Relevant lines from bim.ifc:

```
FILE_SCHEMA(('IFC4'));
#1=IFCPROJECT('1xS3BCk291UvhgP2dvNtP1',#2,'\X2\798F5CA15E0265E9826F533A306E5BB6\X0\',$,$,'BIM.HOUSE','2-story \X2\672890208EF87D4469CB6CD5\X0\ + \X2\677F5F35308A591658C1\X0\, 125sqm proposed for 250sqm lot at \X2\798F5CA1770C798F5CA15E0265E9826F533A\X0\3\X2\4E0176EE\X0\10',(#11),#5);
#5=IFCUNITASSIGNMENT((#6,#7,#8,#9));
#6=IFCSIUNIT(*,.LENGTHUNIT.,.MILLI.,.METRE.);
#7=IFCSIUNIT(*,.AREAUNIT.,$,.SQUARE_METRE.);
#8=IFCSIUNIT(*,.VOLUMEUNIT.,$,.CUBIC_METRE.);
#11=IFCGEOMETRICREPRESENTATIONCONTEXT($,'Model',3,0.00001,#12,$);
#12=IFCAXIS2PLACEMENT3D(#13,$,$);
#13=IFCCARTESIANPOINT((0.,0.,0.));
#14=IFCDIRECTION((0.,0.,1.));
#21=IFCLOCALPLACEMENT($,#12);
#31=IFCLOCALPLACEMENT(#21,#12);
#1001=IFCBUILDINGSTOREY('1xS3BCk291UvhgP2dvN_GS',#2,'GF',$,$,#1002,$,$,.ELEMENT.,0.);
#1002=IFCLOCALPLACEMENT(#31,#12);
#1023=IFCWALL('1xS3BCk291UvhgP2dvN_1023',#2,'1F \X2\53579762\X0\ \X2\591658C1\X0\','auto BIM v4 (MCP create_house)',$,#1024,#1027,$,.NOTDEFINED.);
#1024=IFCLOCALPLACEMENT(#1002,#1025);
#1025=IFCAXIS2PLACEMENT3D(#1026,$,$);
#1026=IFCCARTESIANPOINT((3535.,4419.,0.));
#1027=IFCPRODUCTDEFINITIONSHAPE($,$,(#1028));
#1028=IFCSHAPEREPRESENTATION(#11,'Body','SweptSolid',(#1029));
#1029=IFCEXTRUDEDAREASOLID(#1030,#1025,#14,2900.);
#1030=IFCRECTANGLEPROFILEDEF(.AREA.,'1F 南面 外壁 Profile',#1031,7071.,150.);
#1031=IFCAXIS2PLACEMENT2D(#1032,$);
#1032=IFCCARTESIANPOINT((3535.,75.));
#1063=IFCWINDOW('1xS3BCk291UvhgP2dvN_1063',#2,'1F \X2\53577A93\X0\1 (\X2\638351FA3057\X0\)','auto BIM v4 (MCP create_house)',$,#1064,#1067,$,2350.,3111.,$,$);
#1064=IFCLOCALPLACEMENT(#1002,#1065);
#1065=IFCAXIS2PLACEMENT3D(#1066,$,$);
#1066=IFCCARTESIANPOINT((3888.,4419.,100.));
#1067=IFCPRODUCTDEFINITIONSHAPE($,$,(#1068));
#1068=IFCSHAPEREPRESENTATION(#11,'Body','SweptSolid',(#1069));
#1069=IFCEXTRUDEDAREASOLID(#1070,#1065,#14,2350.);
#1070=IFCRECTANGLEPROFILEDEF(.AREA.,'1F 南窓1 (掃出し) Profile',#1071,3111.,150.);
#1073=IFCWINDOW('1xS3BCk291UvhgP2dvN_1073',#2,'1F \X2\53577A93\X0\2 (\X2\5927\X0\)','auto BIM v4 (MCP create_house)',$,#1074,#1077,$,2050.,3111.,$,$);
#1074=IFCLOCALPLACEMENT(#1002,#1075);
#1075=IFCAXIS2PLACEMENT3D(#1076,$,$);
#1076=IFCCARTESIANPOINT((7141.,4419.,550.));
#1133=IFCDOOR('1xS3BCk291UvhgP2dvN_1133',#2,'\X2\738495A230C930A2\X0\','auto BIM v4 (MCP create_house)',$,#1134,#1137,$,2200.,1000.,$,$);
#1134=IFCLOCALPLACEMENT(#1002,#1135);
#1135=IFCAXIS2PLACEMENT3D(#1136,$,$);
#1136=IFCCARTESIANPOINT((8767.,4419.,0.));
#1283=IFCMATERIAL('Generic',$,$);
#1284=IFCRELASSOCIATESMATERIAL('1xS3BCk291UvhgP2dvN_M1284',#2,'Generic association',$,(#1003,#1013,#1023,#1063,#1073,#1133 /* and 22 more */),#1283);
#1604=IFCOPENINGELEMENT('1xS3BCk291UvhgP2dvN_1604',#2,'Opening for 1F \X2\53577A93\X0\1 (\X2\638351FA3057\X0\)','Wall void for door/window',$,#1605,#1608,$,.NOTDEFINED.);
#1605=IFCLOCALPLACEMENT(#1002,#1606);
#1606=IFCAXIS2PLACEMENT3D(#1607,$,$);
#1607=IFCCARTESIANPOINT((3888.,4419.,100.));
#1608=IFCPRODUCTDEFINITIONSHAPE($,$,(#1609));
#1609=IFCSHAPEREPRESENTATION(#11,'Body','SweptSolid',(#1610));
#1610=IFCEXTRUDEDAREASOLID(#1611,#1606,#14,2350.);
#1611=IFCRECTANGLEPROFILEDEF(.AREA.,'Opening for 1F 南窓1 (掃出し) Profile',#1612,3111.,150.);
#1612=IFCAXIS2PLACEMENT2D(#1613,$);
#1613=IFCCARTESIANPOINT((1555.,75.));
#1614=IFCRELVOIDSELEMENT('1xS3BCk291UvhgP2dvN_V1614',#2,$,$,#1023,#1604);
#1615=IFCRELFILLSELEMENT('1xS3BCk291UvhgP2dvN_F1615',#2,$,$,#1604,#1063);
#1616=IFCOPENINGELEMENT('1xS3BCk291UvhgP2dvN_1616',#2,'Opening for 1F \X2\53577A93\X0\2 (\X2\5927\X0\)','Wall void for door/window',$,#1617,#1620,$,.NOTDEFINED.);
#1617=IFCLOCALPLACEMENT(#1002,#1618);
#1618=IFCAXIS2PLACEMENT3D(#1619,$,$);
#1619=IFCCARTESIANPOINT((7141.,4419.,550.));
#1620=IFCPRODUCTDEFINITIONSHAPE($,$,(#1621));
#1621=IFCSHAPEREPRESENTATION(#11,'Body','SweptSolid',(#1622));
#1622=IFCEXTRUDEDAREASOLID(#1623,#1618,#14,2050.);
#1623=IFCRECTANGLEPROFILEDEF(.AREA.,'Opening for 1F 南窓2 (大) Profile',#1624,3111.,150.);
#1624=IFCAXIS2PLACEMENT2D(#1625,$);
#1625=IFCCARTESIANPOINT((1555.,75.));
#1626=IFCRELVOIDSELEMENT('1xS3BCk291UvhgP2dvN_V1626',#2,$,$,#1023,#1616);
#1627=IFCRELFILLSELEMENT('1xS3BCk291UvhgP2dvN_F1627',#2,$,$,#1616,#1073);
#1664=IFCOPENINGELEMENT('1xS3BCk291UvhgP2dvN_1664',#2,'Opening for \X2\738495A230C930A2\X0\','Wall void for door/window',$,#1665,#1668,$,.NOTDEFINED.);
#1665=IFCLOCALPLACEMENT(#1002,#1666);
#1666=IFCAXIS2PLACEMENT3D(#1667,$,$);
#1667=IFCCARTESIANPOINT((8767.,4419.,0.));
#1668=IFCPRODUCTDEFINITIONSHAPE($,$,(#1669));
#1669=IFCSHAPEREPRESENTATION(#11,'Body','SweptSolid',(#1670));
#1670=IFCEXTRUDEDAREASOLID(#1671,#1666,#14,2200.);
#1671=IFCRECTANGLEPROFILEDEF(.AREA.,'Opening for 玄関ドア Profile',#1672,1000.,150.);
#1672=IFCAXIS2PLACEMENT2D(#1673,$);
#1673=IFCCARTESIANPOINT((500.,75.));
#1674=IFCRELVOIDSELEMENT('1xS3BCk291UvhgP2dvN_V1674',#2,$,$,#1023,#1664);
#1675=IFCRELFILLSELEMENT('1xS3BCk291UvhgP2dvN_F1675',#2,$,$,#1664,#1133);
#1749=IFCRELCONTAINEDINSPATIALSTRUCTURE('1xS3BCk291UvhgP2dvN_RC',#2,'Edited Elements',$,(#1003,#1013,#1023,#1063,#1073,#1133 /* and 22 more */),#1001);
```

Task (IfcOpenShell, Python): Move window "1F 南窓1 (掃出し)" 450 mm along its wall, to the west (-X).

```python
import ifcopenshell
import ifcopenshell.api.geometry
import ifcopenshell.util.placement
import ifcopenshell.util.unit

model = ifcopenshell.open("bim.ifc")
unit_scale = ifcopenshell.util.unit.calculate_unit_scale(model)

window = model.by_id(1063)
opening = window.FillsVoids[0].RelatingOpeningElement
wall = opening.VoidsElements[0].RelatingBuildingElement

wall_matrix = ifcopenshell.util.placement.get_local_placement(wall.ObjectPlacement)
shift = wall_matrix[:3, 0] * -0.45 / unit_scale
before = ifcopenshell.util.placement.get_local_placement(window.ObjectPlacement)[:3, 3].copy()

# The window is not placed relative to its opening, so move both.
for product in (opening, window):
    matrix = ifcopenshell.util.placement.get_local_placement(product.ObjectPlacement)
    matrix[:3, 3] += shift
    ifcopenshell.api.geometry.edit_object_placement(model, product=product, matrix=matrix, is_si=False)

after = ifcopenshell.util.placement.get_local_placement(window.ObjectPlacement)[:3, 3]
print("window moved by", (after - before).round(3) + 0.0)

model.write("bim_edited.ifc")
```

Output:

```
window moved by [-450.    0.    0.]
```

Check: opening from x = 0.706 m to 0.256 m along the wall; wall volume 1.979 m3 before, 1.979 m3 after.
